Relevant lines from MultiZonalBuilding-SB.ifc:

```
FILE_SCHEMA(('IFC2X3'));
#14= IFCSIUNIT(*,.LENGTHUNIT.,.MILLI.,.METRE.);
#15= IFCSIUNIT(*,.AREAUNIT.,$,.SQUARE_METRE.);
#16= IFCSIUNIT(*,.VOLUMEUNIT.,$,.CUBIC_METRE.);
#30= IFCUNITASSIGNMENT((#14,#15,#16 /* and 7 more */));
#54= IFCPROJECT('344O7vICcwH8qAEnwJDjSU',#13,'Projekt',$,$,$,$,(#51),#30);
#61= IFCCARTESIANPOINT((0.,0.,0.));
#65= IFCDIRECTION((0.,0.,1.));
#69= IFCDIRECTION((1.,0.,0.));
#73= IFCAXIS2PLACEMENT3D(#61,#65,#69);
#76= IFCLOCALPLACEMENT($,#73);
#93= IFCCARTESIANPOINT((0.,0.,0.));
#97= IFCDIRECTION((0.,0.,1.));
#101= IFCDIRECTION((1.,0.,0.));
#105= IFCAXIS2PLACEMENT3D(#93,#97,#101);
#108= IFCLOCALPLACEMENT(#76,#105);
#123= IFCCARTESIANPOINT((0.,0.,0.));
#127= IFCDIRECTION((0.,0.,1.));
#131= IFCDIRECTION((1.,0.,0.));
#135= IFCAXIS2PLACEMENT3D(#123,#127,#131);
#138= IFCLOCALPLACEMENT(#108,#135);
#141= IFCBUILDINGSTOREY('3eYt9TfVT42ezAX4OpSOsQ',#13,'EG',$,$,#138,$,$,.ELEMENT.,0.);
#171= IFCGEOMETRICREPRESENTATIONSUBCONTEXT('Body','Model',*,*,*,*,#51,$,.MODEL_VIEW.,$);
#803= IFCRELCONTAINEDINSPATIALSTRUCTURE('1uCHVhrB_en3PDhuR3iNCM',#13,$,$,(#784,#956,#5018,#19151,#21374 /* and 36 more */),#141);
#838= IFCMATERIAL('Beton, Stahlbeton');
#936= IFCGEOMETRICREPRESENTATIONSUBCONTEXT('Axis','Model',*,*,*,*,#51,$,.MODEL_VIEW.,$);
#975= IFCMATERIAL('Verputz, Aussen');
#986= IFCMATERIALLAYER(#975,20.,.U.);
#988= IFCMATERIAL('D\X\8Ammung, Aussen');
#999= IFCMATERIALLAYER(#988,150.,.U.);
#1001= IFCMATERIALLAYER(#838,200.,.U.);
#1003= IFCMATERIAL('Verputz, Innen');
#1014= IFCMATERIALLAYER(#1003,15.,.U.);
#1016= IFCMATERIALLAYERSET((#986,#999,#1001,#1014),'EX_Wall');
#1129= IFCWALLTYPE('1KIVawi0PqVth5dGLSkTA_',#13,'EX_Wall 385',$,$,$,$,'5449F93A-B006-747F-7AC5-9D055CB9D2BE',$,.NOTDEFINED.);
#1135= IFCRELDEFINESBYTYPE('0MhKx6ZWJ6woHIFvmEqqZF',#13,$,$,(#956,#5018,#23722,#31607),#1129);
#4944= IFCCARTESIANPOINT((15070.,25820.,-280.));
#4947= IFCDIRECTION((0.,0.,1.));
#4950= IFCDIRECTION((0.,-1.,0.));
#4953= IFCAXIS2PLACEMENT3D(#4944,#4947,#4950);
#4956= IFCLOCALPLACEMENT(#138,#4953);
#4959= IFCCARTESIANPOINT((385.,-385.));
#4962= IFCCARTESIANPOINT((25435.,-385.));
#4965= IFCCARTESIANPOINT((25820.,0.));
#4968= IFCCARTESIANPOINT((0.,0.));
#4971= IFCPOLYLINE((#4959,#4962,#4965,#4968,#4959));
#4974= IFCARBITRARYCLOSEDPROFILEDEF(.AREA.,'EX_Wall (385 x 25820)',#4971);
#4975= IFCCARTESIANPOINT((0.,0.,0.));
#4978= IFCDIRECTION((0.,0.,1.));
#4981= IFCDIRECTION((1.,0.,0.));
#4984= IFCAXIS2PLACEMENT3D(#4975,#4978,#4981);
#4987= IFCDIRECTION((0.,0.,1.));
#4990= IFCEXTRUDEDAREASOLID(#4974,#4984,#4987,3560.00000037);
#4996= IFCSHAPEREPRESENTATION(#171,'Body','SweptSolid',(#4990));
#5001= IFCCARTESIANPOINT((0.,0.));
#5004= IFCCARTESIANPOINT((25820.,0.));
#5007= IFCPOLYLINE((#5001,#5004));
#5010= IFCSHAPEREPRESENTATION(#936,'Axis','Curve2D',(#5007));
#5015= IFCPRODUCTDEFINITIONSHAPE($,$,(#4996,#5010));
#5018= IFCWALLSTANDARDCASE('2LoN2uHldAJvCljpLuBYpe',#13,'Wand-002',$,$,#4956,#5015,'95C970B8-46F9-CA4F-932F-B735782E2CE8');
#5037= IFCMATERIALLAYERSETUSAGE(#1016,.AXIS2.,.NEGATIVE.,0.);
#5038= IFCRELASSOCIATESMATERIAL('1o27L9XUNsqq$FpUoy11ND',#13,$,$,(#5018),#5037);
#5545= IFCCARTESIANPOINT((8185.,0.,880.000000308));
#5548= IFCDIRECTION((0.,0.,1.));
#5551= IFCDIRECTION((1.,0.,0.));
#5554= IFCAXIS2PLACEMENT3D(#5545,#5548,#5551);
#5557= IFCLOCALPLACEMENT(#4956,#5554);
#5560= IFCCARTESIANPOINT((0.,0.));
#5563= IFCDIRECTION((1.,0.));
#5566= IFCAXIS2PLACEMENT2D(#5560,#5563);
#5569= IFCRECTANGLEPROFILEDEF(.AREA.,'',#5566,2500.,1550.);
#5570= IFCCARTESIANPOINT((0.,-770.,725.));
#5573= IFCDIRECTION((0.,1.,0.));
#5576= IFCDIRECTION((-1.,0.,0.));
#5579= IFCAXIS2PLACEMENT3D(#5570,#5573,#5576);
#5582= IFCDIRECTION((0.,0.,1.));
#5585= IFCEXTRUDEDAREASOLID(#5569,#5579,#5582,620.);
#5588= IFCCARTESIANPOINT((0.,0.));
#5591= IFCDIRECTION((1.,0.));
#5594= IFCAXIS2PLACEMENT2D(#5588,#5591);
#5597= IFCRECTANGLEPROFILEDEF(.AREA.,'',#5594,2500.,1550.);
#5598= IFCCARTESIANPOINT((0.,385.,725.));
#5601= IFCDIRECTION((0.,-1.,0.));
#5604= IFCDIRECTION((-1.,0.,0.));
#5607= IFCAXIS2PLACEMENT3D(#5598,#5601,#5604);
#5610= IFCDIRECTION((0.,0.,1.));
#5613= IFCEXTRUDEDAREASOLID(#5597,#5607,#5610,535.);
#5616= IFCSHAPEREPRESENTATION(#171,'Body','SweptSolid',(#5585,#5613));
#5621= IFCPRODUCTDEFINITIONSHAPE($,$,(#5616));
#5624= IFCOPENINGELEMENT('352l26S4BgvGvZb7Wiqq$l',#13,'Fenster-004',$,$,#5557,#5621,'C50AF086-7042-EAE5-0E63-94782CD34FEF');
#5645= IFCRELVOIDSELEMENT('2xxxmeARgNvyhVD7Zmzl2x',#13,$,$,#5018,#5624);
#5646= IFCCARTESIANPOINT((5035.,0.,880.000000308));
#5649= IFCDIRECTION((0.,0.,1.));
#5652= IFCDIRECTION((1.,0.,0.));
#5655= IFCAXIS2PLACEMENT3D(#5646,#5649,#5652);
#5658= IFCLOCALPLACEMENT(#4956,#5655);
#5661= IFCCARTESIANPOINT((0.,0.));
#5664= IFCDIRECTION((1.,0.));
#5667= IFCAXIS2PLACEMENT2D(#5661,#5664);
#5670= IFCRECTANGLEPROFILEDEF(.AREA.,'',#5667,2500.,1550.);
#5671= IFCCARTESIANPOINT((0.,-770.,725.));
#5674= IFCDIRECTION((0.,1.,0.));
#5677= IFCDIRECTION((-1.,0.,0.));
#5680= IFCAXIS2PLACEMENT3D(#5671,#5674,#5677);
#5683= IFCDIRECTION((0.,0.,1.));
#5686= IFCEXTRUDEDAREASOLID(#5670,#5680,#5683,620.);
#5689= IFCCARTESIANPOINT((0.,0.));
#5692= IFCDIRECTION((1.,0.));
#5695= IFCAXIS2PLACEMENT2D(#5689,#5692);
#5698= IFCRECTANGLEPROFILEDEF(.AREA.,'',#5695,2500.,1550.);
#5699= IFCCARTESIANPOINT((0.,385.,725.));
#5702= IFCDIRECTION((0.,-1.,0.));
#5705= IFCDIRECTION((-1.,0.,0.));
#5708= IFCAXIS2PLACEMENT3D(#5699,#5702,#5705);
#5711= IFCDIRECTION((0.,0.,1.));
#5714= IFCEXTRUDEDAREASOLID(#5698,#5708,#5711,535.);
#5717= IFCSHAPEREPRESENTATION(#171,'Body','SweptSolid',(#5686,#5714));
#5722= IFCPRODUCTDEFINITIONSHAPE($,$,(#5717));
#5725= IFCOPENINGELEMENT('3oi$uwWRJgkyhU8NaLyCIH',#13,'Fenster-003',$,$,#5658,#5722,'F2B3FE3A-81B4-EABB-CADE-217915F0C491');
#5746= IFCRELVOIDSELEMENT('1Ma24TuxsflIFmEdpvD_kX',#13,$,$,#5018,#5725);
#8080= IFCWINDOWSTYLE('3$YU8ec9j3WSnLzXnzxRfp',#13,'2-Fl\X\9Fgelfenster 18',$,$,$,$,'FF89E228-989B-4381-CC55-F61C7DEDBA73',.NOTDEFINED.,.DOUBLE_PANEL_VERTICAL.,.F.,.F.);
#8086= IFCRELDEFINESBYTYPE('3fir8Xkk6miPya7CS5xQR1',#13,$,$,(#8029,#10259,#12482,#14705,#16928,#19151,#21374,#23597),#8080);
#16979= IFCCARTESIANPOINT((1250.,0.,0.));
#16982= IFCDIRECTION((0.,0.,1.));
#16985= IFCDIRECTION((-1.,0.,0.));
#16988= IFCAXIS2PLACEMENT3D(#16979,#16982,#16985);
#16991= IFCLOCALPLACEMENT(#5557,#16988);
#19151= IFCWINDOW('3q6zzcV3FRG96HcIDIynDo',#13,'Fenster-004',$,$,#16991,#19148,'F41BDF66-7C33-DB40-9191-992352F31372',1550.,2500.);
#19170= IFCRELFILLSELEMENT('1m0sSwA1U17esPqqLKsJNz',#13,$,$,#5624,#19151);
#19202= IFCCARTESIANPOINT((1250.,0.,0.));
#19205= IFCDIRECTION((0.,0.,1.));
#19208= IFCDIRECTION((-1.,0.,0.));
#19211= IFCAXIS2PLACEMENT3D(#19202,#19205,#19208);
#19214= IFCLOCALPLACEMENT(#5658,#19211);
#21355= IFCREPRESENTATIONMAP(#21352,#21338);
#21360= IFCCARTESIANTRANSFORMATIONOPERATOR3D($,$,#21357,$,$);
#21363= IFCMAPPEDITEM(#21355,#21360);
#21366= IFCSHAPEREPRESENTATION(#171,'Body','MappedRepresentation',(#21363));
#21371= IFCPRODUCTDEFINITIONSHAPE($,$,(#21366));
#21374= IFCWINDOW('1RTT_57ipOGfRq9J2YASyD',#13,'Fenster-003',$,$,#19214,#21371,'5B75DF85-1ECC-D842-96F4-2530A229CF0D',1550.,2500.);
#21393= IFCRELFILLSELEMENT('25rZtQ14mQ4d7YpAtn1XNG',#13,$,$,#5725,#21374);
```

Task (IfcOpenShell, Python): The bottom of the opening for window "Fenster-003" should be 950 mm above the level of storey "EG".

```python
import numpy as np
import ifcopenshell
import ifcopenshell.api.geometry
import ifcopenshell.geom
import ifcopenshell.util.element
import ifcopenshell.util.placement
import ifcopenshell.util.shape
import ifcopenshell.util.unit

model = ifcopenshell.open("MultiZonalBuilding-SB.ifc")
unit_scale = ifcopenshell.util.unit.calculate_unit_scale(model)

window = model.by_guid("1RTT_57ipOGfRq9J2YASyD")
opening = window.FillsVoids[0].RelatingOpeningElement
storey = ifcopenshell.util.element.get_container(window, ifc_class="IfcBuildingStorey")
level = ifcopenshell.util.placement.get_local_placement(storey.ObjectPlacement)[2, 3]

# The opening's origin need not be at the sill, so measure its lowest point.
shape = ifcopenshell.geom.create_shape(ifcopenshell.geom.settings(), opening)
bottom = ifcopenshell.util.shape.get_shape_bottom_elevation(shape, shape.geometry) / unit_scale
dz = level + 0.95 / unit_scale - bottom

shift = np.array([0.0, 0.0, dz])
# The window is placed relative to its opening, so it follows when the opening moves.
matrix = ifcopenshell.util.placement.get_local_placement(opening.ObjectPlacement)
matrix[:3, 3] += shift
ifcopenshell.api.geometry.edit_object_placement(
    model, product=opening, matrix=matrix, is_si=False, should_transform_children=True
)

print(f"moved by {dz * unit_scale:+.3f} m")

model.write("MultiZonalBuilding-SB_edited.ifc")
```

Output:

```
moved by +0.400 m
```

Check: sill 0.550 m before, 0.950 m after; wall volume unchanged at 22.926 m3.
